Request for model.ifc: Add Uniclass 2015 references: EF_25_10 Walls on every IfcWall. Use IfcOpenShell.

First a look at what the model holds.

```python
import ifcopenshell

model = ifcopenshell.open("model.ifc")
print(model.schema)
print("classifications:", [c.Name for c in model.by_type("IfcClassification")])
for ifc_class in ("IfcDoor", "IfcRoof", "IfcStair", "IfcWall", "IfcWindow"):
    print(ifc_class, len(model.by_type(ifc_class)))
```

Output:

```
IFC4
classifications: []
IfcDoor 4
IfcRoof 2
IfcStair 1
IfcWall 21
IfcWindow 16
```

```python
import ifcopenshell
import ifcopenshell.api.classification

model = ifcopenshell.open("model.ifc")

system = ifcopenshell.api.classification.add_classification(model, classification="Uniclass 2015")

codes = {
    "IfcWall": ("EF_25_10", "Walls"),
}
for ifc_class, (code, name) in codes.items():
    products = model.by_type(ifc_class)
    ifcopenshell.api.classification.add_reference(
        model, products=products, classification=system, identification=code, name=name
    )
    print(code, len(products))

model.write("model-out.ifc")
```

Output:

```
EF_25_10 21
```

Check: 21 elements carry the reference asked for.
